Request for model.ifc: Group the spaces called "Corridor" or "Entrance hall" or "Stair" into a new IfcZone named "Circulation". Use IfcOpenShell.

First a look at what the model holds.

```python
import ifcopenshell

model = ifcopenshell.open("model.ifc")
print(model.schema)
seen = {}
for space in model.by_type("IfcSpace"):
    seen[space.LongName] = seen.get(space.LongName, 0) + 1
for name, count in sorted(seen.items(), key=str):
    print(count, "x", name)
print("zones:", [z.Name for z in model.by_type("IfcZone")][:20])
```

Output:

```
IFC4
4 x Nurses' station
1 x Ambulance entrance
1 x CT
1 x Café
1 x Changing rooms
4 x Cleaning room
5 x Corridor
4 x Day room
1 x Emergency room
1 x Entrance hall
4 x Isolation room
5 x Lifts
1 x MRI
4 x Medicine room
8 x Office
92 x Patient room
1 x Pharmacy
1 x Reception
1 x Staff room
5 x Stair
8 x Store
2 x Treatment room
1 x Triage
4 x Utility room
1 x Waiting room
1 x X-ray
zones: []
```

```python
import ifcopenshell
import ifcopenshell.api.group
import ifcopenshell.api.root

model = ifcopenshell.open("model.ifc")

names = {"Corridor", "Entrance hall", "Stair"}
spaces = [s for s in model.by_type("IfcSpace") if s.LongName in names]

zone = ifcopenshell.api.root.create_entity(model, ifc_class="IfcZone", name="Circulation")
ifcopenshell.api.group.assign_group(model, products=spaces, group=zone)
print(len(spaces), "spaces in", zone.Name)

model.write("model_v2.ifc")
```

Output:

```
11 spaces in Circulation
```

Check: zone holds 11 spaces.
